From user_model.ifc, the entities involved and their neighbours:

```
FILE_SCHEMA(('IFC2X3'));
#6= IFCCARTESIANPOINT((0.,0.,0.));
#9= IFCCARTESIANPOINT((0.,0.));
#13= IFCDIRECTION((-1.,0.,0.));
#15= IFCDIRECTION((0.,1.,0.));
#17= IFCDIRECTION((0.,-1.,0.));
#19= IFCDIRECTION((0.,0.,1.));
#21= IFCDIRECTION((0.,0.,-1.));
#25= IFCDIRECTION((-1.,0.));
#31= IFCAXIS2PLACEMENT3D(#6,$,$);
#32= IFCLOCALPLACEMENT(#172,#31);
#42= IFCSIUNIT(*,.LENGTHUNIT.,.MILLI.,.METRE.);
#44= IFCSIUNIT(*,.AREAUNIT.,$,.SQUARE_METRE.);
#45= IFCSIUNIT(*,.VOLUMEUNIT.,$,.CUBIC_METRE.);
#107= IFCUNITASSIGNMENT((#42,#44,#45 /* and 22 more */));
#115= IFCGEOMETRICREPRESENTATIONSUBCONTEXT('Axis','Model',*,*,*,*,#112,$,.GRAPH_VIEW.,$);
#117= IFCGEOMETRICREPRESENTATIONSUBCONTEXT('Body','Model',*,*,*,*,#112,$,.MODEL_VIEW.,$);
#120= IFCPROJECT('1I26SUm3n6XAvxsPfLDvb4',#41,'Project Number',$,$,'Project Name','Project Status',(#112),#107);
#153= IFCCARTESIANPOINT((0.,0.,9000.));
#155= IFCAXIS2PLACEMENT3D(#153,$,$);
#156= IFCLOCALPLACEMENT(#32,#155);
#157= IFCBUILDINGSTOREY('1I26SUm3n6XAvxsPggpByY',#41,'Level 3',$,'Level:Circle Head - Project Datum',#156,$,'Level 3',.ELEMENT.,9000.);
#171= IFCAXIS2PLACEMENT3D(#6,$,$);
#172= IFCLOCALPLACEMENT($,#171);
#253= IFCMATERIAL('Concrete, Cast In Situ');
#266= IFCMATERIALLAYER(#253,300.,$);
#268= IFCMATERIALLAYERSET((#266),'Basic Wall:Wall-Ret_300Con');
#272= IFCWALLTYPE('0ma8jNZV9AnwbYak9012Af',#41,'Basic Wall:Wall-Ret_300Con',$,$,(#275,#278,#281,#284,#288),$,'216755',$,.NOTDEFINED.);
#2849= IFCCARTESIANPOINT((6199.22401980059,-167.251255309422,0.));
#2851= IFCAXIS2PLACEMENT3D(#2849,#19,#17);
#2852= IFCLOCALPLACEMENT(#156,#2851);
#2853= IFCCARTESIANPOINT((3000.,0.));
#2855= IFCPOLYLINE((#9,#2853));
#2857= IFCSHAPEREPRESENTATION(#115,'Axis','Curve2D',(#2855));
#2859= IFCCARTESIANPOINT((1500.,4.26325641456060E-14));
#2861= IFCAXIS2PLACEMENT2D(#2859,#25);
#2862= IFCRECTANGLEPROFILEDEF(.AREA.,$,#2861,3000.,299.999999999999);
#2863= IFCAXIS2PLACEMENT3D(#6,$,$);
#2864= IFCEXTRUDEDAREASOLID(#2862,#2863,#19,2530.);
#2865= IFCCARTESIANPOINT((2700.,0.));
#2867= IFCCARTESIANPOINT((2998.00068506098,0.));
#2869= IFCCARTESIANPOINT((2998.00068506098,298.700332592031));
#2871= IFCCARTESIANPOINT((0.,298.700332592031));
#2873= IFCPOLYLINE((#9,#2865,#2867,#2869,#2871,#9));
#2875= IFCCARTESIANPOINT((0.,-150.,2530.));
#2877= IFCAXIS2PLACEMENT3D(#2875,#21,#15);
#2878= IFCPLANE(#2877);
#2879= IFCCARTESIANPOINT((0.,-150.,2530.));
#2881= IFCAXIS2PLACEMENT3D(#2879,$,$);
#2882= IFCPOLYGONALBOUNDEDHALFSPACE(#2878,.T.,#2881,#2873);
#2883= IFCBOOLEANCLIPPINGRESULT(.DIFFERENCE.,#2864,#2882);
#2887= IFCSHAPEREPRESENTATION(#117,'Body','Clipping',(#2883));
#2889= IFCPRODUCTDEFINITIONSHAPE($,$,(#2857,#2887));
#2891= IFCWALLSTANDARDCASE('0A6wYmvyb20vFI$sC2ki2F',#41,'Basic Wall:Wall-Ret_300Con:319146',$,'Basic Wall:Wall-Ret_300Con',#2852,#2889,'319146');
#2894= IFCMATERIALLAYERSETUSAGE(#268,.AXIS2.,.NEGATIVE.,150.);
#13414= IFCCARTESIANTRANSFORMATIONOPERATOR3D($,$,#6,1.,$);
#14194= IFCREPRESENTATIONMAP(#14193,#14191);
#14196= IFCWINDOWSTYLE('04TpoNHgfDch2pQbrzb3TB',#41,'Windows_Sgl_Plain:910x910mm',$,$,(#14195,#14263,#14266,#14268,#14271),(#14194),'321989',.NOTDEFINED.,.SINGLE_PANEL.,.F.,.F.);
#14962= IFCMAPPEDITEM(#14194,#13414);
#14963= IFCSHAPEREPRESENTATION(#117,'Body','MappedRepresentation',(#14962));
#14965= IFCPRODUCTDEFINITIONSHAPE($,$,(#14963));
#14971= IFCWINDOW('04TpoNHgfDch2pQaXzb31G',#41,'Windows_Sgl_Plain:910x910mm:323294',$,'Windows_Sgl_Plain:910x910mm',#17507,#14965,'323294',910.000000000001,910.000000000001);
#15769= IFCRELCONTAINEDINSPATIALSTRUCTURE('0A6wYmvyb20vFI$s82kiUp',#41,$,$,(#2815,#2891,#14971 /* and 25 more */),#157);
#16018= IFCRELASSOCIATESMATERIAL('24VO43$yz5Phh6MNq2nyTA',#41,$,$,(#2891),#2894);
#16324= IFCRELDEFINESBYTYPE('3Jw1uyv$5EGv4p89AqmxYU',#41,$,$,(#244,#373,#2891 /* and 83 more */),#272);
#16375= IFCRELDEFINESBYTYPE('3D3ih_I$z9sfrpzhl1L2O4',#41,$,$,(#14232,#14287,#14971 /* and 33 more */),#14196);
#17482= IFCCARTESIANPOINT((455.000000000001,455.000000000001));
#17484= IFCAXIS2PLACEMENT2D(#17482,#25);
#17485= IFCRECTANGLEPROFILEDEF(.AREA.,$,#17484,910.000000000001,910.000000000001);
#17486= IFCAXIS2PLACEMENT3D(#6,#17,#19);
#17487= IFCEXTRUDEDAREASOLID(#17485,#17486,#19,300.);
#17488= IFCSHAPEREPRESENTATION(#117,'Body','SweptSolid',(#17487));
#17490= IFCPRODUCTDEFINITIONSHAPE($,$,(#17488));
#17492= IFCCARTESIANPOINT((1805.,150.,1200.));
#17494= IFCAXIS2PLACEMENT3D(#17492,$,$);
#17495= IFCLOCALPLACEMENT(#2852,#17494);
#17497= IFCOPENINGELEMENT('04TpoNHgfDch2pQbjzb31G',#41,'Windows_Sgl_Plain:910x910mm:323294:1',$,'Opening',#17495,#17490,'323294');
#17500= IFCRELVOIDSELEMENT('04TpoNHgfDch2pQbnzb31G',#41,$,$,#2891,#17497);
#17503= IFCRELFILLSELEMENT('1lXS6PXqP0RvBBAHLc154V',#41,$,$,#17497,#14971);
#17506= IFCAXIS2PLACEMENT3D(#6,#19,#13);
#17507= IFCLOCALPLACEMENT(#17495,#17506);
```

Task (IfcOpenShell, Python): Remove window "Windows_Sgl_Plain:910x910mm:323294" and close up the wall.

```python
import ifcopenshell
import ifcopenshell.api.feature
import ifcopenshell.api.root
import ifcopenshell.geom
import ifcopenshell.util.shape

model = ifcopenshell.open("user_model.ifc")
settings = ifcopenshell.geom.settings()


def volume(element):
    """Net volume in cubic metres, openings subtracted."""
    shape = ifcopenshell.geom.create_shape(settings, element)
    return ifcopenshell.util.shape.get_volume(shape.geometry)


window = model.by_guid("04TpoNHgfDch2pQaXzb31G")
opening = window.FillsVoids[0].RelatingOpeningElement
wall = opening.VoidsElements[0].RelatingBuildingElement
before = volume(wall)

ifcopenshell.api.root.remove_product(model, product=window)
ifcopenshell.api.feature.remove_feature(model, feature=opening)

after = volume(wall)

print(f"wall volume {before:.3f} -> {after:.3f} m3")

model.write("user_model_edited.ifc")
```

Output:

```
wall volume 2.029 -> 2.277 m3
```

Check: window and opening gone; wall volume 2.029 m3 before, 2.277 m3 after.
